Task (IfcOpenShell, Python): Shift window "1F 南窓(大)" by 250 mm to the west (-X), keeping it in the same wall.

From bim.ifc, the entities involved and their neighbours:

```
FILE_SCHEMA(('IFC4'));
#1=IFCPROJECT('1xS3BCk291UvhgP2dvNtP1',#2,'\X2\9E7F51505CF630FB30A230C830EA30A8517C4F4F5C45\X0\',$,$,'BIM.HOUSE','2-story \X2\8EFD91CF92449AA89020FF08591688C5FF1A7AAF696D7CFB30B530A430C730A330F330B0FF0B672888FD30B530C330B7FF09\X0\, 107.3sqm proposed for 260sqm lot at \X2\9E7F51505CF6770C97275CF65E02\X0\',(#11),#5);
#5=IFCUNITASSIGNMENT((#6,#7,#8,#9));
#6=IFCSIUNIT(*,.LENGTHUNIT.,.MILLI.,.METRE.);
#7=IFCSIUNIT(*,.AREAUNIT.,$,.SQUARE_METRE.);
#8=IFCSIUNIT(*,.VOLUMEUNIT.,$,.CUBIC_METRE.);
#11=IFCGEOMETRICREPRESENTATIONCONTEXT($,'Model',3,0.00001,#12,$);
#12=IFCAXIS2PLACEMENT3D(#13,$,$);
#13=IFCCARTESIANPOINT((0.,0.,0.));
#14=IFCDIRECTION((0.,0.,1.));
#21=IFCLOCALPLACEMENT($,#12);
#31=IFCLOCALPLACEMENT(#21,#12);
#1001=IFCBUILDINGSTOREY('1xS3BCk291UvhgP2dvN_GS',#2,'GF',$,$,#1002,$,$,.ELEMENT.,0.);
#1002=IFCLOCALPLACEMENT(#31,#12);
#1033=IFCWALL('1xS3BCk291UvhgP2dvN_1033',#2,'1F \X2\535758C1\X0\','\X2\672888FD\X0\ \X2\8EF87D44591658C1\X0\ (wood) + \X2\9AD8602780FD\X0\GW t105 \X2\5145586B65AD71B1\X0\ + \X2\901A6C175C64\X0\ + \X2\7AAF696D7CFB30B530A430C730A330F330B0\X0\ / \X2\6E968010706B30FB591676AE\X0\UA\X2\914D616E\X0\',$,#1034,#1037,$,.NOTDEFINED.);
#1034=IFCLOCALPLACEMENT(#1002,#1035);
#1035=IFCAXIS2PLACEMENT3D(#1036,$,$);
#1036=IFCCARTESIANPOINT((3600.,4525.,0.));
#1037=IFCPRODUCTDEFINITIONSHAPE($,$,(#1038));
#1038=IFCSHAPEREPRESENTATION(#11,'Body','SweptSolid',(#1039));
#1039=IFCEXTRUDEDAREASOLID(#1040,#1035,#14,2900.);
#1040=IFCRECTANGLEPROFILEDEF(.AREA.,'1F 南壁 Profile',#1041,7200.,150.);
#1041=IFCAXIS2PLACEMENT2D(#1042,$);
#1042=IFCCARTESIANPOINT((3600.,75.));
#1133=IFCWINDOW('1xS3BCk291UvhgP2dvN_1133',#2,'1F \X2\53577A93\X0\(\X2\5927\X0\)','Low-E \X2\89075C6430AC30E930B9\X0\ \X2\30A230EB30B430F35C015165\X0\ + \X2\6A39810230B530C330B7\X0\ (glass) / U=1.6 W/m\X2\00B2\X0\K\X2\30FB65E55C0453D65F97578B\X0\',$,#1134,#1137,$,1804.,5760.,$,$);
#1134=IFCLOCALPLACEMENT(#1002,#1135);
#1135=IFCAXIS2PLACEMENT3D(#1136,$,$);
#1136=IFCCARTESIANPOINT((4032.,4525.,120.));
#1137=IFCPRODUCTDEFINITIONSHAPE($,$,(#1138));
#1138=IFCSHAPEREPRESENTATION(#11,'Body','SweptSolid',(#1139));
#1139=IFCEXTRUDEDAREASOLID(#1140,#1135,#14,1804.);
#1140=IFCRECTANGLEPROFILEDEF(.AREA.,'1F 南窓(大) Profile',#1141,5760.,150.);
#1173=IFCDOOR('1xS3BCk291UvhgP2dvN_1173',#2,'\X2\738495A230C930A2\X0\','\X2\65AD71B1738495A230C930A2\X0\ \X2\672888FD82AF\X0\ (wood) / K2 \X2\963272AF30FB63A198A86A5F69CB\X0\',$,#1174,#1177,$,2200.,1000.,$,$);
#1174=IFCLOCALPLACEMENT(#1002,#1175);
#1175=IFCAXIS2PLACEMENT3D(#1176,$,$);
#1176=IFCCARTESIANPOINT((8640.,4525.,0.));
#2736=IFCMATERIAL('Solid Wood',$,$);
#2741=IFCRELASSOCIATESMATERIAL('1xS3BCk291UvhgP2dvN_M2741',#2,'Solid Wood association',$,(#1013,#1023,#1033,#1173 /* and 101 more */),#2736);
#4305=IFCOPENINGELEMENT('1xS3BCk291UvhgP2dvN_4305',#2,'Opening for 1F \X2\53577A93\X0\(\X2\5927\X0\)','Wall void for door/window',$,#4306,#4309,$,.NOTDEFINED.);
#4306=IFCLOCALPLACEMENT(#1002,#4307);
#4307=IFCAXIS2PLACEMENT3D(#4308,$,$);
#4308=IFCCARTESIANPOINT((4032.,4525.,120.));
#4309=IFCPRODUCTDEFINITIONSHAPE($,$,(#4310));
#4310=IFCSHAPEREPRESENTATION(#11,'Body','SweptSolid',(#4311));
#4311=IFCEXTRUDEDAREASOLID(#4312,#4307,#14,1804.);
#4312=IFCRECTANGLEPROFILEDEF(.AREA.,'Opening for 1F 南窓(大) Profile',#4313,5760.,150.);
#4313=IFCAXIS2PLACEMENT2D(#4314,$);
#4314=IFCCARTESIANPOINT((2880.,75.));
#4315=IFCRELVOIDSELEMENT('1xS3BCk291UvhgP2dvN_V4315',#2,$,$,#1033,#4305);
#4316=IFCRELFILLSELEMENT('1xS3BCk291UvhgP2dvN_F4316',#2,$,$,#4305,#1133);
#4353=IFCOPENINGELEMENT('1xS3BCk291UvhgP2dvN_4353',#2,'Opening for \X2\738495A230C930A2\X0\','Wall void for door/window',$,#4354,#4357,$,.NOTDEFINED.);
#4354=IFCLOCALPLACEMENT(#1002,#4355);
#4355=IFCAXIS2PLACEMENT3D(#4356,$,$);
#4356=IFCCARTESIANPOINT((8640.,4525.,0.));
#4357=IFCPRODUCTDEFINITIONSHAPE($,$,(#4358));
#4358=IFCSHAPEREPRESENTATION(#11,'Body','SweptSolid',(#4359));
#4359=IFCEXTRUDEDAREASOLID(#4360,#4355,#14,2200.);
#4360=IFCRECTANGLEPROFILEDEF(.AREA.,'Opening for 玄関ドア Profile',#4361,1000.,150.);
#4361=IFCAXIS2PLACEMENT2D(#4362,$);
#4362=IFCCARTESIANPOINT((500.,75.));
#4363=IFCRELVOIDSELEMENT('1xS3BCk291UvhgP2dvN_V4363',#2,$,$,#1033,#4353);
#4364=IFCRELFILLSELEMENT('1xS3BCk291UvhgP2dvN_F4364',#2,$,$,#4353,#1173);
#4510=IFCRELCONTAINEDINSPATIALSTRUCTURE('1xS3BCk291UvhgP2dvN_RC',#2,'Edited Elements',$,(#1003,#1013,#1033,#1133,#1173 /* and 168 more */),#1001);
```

```python
import ifcopenshell
import ifcopenshell.api.geometry
import ifcopenshell.util.placement
import ifcopenshell.util.unit

model = ifcopenshell.open("bim.ifc")
unit_scale = ifcopenshell.util.unit.calculate_unit_scale(model)

window = model.by_id(1133)
opening = window.FillsVoids[0].RelatingOpeningElement
wall = opening.VoidsElements[0].RelatingBuildingElement

wall_matrix = ifcopenshell.util.placement.get_local_placement(wall.ObjectPlacement)
shift = wall_matrix[:3, 0] * -0.25 / unit_scale
before = ifcopenshell.util.placement.get_local_placement(window.ObjectPlacement)[:3, 3].copy()

# The window is not placed relative to its opening, so move both.
for product in (opening, window):
    matrix = ifcopenshell.util.placement.get_local_placement(product.ObjectPlacement)
    matrix[:3, 3] += shift
    ifcopenshell.api.geometry.edit_object_placement(model, product=product, matrix=matrix, is_si=False)

after = ifcopenshell.util.placement.get_local_placement(window.ObjectPlacement)[:3, 3]
print("window moved by", (after - before).round(3) + 0.0)

model.write("bim_updated.ifc")
```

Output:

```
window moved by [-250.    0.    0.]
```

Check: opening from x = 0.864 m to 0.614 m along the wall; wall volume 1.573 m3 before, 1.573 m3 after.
